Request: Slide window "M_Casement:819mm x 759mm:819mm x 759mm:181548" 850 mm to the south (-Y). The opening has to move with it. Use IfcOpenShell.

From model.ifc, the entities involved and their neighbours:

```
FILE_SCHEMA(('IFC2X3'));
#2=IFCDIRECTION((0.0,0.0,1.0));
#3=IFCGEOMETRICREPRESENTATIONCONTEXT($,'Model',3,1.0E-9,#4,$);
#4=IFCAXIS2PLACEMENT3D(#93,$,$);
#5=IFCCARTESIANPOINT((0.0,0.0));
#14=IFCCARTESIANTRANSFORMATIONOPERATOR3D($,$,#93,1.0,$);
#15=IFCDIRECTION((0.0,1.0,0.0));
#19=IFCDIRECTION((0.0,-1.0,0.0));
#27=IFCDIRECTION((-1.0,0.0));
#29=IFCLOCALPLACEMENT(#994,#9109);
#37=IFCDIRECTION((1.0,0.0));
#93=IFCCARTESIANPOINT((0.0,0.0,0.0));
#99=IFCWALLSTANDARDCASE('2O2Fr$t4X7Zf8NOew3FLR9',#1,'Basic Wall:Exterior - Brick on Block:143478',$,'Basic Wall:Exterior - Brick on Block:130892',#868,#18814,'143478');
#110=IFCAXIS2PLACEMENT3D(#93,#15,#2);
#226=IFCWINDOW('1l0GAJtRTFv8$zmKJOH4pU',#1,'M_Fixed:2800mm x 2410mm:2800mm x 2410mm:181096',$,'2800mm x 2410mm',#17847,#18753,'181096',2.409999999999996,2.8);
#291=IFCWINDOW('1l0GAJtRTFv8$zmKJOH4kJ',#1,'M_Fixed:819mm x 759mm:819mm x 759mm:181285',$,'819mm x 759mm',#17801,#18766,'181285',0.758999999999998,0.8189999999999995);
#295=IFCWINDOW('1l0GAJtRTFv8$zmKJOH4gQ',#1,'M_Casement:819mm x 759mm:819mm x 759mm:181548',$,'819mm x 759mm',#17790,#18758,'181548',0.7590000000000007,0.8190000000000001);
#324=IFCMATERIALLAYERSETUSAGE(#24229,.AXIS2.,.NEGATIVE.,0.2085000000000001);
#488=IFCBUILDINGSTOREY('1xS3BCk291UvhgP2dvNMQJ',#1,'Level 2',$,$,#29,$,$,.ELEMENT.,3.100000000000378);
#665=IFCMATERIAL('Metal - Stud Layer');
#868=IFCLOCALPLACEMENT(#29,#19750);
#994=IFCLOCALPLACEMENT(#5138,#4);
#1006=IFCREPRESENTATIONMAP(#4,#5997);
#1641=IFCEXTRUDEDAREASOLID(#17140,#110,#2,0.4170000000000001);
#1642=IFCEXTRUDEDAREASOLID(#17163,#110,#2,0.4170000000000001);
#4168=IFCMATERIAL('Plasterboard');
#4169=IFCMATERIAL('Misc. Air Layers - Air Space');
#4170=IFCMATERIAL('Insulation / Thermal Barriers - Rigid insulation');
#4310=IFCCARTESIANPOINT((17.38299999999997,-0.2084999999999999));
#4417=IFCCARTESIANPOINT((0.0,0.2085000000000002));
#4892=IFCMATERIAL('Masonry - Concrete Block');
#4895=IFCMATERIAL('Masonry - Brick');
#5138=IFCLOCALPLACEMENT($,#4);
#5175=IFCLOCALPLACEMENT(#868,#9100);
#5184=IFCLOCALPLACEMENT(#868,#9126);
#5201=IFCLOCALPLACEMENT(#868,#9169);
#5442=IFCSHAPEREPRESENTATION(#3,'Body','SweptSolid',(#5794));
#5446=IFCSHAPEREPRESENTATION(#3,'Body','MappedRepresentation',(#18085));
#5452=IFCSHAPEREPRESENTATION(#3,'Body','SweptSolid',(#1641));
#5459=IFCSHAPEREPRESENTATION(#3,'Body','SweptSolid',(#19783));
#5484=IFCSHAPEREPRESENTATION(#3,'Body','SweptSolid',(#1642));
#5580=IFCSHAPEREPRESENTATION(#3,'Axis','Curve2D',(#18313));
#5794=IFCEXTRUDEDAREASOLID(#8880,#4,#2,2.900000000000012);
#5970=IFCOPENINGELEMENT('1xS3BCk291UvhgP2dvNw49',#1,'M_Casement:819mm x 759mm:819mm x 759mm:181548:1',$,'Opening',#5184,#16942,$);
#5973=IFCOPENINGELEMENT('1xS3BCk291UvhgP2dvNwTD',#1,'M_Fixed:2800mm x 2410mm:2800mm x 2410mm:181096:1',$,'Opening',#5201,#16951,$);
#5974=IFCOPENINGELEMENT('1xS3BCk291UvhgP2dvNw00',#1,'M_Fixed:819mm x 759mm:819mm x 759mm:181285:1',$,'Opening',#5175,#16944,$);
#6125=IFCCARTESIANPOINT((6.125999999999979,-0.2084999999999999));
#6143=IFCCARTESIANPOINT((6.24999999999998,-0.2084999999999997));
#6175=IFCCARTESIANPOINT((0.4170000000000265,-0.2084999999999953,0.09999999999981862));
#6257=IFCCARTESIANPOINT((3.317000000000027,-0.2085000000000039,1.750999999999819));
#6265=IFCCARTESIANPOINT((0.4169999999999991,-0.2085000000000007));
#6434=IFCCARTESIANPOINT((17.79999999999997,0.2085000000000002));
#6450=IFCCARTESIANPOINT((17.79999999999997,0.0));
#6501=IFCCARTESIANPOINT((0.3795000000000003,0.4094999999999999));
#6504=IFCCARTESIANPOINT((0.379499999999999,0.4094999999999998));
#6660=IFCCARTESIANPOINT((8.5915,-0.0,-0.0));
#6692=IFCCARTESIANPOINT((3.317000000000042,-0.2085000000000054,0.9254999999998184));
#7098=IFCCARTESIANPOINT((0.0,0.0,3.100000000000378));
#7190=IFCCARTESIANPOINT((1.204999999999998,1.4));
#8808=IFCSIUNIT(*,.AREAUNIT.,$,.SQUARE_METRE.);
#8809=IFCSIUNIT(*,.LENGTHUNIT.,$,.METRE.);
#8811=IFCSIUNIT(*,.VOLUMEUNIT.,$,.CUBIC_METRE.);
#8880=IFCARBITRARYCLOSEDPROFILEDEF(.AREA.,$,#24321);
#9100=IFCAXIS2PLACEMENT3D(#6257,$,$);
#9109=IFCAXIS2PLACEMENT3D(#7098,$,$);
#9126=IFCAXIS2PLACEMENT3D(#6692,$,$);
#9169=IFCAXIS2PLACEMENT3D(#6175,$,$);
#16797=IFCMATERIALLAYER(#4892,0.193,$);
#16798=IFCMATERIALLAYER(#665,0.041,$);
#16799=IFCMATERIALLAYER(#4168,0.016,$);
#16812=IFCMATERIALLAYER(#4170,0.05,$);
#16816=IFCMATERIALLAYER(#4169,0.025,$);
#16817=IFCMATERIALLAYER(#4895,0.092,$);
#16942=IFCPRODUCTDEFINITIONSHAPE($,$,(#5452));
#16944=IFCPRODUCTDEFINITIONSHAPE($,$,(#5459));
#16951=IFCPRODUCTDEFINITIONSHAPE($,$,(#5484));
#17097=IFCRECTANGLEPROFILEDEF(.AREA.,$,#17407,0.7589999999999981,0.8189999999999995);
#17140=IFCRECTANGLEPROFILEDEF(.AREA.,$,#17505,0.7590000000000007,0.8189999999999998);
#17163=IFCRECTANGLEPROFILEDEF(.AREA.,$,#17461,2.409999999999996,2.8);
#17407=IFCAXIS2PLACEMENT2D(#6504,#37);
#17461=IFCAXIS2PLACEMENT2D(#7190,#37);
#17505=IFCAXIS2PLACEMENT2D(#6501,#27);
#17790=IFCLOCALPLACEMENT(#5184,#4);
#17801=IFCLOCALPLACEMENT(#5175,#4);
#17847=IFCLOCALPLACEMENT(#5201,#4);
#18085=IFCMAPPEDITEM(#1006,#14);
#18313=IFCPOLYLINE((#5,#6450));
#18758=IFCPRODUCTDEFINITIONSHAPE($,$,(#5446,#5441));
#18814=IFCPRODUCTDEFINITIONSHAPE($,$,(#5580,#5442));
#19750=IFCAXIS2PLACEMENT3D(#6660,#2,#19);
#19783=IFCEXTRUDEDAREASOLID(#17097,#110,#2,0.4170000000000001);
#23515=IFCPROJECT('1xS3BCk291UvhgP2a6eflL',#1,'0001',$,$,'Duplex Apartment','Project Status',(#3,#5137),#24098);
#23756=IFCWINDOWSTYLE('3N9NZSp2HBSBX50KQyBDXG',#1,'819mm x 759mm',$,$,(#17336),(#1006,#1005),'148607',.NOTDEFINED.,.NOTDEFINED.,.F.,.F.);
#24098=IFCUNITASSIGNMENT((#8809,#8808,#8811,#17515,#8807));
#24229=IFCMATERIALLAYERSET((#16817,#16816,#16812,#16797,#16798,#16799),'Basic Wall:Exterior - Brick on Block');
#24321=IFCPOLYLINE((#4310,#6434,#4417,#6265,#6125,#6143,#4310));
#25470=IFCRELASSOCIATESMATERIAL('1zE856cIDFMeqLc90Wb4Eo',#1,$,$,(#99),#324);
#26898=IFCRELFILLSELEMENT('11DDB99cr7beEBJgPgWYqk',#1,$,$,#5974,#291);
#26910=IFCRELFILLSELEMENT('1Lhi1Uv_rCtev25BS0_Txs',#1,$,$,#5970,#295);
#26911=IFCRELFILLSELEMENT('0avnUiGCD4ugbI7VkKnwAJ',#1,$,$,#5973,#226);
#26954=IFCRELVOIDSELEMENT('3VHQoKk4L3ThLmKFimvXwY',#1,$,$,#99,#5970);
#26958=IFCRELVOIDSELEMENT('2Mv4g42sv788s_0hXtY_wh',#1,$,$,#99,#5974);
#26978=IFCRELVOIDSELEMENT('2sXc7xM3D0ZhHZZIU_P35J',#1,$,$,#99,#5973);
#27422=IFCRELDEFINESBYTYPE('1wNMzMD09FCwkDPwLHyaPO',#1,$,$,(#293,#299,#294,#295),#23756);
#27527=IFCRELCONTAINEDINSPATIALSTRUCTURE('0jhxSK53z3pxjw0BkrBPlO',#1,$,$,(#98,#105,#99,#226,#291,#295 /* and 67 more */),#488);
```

```python
import ifcopenshell
import ifcopenshell.api.geometry
import ifcopenshell.util.placement
import ifcopenshell.util.unit

model = ifcopenshell.open("model.ifc")
unit_scale = ifcopenshell.util.unit.calculate_unit_scale(model)

window = model.by_id(295)
opening = window.FillsVoids[0].RelatingOpeningElement
wall = opening.VoidsElements[0].RelatingBuildingElement

wall_matrix = ifcopenshell.util.placement.get_local_placement(wall.ObjectPlacement)
shift = wall_matrix[:3, 0] * 0.85 / unit_scale
before = ifcopenshell.util.placement.get_local_placement(window.ObjectPlacement)[:3, 3].copy()

# The window is placed relative to its opening, so it follows when the opening moves.
matrix = ifcopenshell.util.placement.get_local_placement(opening.ObjectPlacement)
matrix[:3, 3] += shift
ifcopenshell.api.geometry.edit_object_placement(
    model, product=opening, matrix=matrix, is_si=False, should_transform_children=True
)

after = ifcopenshell.util.placement.get_local_placement(window.ObjectPlacement)[:3, 3]
print("window moved by", (after - before).round(3) + 0.0)

model.write("model_rev.ifc")
```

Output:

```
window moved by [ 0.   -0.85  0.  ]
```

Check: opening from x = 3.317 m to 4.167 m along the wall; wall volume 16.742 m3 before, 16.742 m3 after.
